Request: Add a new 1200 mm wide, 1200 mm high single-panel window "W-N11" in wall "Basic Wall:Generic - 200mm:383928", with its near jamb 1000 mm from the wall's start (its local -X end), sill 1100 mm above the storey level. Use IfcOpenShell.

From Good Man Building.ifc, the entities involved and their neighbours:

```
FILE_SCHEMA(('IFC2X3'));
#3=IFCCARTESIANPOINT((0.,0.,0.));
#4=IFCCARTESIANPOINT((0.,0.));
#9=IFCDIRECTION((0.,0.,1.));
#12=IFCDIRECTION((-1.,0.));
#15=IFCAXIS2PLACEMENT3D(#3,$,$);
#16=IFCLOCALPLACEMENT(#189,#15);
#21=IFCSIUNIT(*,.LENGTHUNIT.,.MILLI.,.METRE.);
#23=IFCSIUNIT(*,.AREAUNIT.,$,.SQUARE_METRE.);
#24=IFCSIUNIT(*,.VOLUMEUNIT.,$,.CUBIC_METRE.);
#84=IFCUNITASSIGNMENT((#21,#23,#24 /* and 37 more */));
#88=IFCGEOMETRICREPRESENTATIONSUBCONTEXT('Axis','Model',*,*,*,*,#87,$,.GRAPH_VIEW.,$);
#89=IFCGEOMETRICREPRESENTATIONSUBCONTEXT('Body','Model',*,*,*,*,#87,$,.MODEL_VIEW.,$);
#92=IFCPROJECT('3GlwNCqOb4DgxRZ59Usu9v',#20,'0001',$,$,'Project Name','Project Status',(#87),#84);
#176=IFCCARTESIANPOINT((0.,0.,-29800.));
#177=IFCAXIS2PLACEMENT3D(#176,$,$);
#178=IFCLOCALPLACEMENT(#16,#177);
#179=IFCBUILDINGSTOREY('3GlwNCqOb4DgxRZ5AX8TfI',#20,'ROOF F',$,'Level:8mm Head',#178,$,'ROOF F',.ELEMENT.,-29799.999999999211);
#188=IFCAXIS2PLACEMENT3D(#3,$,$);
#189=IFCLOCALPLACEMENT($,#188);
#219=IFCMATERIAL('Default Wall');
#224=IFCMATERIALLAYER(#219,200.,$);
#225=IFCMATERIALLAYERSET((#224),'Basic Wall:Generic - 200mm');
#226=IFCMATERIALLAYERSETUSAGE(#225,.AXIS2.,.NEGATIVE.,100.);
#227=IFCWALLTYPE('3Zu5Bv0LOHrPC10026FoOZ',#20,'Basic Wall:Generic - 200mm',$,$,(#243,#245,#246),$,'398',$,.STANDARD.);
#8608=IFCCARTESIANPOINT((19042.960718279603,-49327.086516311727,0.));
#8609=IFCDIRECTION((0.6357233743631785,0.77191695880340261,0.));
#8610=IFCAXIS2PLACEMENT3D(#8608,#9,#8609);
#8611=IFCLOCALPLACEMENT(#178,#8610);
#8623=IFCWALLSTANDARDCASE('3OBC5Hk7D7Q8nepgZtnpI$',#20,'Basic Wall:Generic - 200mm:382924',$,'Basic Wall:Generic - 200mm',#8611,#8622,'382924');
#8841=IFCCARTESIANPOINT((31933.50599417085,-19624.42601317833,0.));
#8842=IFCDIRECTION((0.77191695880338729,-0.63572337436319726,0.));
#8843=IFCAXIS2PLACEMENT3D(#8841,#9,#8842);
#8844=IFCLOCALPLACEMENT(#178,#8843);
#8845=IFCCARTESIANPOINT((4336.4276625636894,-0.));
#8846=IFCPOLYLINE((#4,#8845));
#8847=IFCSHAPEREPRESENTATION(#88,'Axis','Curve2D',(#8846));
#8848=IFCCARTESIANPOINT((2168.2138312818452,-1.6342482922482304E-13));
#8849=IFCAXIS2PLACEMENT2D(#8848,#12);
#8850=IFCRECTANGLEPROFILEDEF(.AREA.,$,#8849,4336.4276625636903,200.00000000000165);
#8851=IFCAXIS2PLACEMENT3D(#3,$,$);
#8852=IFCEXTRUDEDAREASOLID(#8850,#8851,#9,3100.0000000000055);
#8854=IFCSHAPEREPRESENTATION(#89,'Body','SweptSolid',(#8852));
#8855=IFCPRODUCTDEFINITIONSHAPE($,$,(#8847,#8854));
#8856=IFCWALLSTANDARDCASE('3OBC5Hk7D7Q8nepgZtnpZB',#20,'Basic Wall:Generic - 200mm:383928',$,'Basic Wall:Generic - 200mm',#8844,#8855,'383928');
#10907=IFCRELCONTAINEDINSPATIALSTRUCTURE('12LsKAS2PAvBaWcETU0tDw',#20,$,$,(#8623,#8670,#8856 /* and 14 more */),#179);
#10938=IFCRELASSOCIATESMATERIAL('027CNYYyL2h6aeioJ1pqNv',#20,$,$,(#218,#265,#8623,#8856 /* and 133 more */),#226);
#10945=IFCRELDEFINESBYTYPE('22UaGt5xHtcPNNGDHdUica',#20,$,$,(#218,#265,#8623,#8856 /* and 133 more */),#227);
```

```python
import numpy as np
import ifcopenshell
import ifcopenshell.api.feature
import ifcopenshell.api.geometry
import ifcopenshell.api.root
import ifcopenshell.api.spatial
import ifcopenshell.api.type
import ifcopenshell.geom
import ifcopenshell.util.element
import ifcopenshell.util.placement
import ifcopenshell.util.representation
import ifcopenshell.util.shape
import ifcopenshell.util.unit

model = ifcopenshell.open("Good Man Building.ifc")
unit_scale = ifcopenshell.util.unit.calculate_unit_scale(model)
settings = ifcopenshell.geom.settings()


def volume(element):
    """Net volume in cubic metres, openings subtracted."""
    shape = ifcopenshell.geom.create_shape(settings, element)
    return ifcopenshell.util.shape.get_volume(shape.geometry)


wall = model.by_guid("3OBC5Hk7D7Q8nepgZtnpZB")
storey = ifcopenshell.util.element.get_container(wall, ifc_class="IfcBuildingStorey")
context = ifcopenshell.util.representation.get_context(model, "Model", "Body", "MODEL_VIEW")
before = volume(wall)

width, height, from_end, sill = 1.2, 1.2, 1, 1.1  # metres

# The wall runs along its own X axis, and the end named is its -X end.
wall_shape = ifcopenshell.geom.create_shape(settings, wall)
x, y, z = ifcopenshell.util.shape.get_vertices(wall_shape.geometry).T
start = x.min() + from_end
face, thickness = float(y.min()), float(y.max() - y.min())
wall_matrix = ifcopenshell.util.placement.get_local_placement(wall.ObjectPlacement)
level = ifcopenshell.util.placement.get_local_placement(storey.ObjectPlacement)[2, 3]


def in_wall(x, y):
    """Placement at x, y metres in the wall's axes, at sill height."""
    matrix = wall_matrix.copy()
    matrix[:, 3] = wall_matrix @ np.array([x / unit_scale, y / unit_scale, 0.0, 1.0])
    matrix[2, 3] = level + sill / unit_scale
    return matrix


# Opening: a box that overshoots both wall faces by 50 mm.
opening = ifcopenshell.api.root.create_entity(model, ifc_class="IfcOpeningElement")
box = ifcopenshell.api.geometry.add_wall_representation(
    model, context=context, length=width, height=height, thickness=thickness + 0.1
)
ifcopenshell.api.geometry.assign_representation(model, product=opening, representation=box)
ifcopenshell.api.geometry.edit_object_placement(model, product=opening, matrix=in_wall(start, face - 0.05), is_si=False)
ifcopenshell.api.feature.add_feature(model, feature=opening, element=wall)

window = ifcopenshell.api.root.create_entity(model, ifc_class="IfcWindow", name="W-N11")
window.OverallWidth, window.OverallHeight = width / unit_scale, height / unit_scale
body = ifcopenshell.api.geometry.add_window_representation(
    model,
    context=context,
    overall_width=window.OverallWidth,
    overall_height=window.OverallHeight,
    partition_type="SINGLE_PANEL",
)
ifcopenshell.api.geometry.assign_representation(model, product=window, representation=body)
ifcopenshell.api.spatial.assign_container(model, products=[window], relating_structure=storey)
fills = ifcopenshell.api.feature.add_filling(model, opening=opening, element=window)
fills.OwnerHistory = window.OwnerHistory  # required in IFC2X3

# IFC2X3 keeps the operation on the window style.
style = ifcopenshell.api.root.create_entity(model, ifc_class="IfcWindowStyle", name="W-N11")
style.OperationType, style.ConstructionType = "SINGLE_PANEL", "NOTDEFINED"
style.ParameterTakesPrecedence = style.Sizeable = False
ifcopenshell.api.type.assign_type(model, related_objects=[window], relating_type=style)

# Centre the window in the wall's thickness.
ifcopenshell.api.geometry.edit_object_placement(model, product=window, matrix=in_wall(start, face), is_si=False)
window_shape = ifcopenshell.geom.create_shape(settings, window)
depth = ifcopenshell.util.shape.get_vertices(window_shape.geometry)[:, 1]
offset = face + thickness / 2 - (depth.min() + depth.max()) / 2
ifcopenshell.api.geometry.edit_object_placement(model, product=window, matrix=in_wall(start, offset), is_si=False)

after = volume(wall)

print(f"wall volume {before:.3f} -> {after:.3f} m3")

model.write("Good Man Building_rev.ifc")
```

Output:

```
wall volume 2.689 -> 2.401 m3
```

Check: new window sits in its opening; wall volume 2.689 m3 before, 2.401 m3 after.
